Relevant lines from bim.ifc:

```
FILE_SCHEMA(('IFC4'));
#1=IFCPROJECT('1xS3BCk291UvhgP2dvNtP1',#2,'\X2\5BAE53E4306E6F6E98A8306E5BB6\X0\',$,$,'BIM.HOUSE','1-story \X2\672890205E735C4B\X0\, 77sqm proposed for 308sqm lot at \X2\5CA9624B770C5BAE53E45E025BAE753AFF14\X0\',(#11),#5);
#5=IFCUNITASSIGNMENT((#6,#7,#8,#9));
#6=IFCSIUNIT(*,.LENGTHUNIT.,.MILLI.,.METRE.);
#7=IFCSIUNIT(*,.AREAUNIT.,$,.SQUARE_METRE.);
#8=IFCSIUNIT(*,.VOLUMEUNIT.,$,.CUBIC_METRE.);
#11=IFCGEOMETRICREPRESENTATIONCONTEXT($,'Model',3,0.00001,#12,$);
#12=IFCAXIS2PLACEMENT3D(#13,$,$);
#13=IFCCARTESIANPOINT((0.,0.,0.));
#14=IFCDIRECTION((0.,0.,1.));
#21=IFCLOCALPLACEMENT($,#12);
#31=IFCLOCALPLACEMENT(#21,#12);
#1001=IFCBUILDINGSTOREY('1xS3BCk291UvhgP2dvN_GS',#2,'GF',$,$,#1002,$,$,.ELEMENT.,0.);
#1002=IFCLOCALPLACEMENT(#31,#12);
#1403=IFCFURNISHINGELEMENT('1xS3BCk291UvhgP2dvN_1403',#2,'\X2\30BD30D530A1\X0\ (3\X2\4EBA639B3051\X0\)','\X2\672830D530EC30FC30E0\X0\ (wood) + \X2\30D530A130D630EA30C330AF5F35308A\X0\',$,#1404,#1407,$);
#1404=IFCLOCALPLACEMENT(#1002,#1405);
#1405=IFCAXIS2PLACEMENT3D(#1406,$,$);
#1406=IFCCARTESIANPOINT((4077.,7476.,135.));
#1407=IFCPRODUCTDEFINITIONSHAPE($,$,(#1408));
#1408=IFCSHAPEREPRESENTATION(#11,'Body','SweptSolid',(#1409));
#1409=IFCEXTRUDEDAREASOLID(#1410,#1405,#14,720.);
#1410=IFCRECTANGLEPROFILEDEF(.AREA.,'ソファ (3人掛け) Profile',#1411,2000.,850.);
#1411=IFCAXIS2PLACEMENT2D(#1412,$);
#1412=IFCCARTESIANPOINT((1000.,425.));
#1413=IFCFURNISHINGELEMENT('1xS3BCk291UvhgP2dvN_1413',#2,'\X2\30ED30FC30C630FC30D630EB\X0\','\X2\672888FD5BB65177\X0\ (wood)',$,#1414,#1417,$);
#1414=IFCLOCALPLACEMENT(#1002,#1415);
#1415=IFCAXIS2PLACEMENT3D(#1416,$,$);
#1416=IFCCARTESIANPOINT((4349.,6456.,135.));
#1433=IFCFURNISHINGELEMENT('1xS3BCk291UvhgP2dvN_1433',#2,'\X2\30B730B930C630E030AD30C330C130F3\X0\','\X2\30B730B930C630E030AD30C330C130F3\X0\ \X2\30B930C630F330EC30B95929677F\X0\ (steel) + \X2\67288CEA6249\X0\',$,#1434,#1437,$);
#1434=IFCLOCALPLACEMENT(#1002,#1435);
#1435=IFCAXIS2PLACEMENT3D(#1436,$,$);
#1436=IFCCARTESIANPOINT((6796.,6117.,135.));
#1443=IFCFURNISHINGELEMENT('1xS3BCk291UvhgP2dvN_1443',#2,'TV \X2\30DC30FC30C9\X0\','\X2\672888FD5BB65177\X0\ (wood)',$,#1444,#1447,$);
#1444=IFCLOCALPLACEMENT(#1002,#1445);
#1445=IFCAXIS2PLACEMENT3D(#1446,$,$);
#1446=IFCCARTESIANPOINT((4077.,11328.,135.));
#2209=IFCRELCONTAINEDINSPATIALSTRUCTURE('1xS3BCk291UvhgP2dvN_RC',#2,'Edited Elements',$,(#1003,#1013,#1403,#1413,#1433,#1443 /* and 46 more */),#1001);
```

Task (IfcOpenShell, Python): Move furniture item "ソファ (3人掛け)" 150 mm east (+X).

```python
import ifcopenshell
import ifcopenshell.api.geometry
import ifcopenshell.util.placement

model = ifcopenshell.open("bim.ifc")

item = model.by_guid("1xS3BCk291UvhgP2dvN_1403")
matrix = ifcopenshell.util.placement.get_local_placement(item.ObjectPlacement)
matrix[0, 3] += 150.0
ifcopenshell.api.geometry.edit_object_placement(model, product=item, matrix=matrix, is_si=False)

print(ifcopenshell.util.placement.get_local_placement(item.ObjectPlacement).round(3) + 0.0)

model.write("bim-out.ifc")
```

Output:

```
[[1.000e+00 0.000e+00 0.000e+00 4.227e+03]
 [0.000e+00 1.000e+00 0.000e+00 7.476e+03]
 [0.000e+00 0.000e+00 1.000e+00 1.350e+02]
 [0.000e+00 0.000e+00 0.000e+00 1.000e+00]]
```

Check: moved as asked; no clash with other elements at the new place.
